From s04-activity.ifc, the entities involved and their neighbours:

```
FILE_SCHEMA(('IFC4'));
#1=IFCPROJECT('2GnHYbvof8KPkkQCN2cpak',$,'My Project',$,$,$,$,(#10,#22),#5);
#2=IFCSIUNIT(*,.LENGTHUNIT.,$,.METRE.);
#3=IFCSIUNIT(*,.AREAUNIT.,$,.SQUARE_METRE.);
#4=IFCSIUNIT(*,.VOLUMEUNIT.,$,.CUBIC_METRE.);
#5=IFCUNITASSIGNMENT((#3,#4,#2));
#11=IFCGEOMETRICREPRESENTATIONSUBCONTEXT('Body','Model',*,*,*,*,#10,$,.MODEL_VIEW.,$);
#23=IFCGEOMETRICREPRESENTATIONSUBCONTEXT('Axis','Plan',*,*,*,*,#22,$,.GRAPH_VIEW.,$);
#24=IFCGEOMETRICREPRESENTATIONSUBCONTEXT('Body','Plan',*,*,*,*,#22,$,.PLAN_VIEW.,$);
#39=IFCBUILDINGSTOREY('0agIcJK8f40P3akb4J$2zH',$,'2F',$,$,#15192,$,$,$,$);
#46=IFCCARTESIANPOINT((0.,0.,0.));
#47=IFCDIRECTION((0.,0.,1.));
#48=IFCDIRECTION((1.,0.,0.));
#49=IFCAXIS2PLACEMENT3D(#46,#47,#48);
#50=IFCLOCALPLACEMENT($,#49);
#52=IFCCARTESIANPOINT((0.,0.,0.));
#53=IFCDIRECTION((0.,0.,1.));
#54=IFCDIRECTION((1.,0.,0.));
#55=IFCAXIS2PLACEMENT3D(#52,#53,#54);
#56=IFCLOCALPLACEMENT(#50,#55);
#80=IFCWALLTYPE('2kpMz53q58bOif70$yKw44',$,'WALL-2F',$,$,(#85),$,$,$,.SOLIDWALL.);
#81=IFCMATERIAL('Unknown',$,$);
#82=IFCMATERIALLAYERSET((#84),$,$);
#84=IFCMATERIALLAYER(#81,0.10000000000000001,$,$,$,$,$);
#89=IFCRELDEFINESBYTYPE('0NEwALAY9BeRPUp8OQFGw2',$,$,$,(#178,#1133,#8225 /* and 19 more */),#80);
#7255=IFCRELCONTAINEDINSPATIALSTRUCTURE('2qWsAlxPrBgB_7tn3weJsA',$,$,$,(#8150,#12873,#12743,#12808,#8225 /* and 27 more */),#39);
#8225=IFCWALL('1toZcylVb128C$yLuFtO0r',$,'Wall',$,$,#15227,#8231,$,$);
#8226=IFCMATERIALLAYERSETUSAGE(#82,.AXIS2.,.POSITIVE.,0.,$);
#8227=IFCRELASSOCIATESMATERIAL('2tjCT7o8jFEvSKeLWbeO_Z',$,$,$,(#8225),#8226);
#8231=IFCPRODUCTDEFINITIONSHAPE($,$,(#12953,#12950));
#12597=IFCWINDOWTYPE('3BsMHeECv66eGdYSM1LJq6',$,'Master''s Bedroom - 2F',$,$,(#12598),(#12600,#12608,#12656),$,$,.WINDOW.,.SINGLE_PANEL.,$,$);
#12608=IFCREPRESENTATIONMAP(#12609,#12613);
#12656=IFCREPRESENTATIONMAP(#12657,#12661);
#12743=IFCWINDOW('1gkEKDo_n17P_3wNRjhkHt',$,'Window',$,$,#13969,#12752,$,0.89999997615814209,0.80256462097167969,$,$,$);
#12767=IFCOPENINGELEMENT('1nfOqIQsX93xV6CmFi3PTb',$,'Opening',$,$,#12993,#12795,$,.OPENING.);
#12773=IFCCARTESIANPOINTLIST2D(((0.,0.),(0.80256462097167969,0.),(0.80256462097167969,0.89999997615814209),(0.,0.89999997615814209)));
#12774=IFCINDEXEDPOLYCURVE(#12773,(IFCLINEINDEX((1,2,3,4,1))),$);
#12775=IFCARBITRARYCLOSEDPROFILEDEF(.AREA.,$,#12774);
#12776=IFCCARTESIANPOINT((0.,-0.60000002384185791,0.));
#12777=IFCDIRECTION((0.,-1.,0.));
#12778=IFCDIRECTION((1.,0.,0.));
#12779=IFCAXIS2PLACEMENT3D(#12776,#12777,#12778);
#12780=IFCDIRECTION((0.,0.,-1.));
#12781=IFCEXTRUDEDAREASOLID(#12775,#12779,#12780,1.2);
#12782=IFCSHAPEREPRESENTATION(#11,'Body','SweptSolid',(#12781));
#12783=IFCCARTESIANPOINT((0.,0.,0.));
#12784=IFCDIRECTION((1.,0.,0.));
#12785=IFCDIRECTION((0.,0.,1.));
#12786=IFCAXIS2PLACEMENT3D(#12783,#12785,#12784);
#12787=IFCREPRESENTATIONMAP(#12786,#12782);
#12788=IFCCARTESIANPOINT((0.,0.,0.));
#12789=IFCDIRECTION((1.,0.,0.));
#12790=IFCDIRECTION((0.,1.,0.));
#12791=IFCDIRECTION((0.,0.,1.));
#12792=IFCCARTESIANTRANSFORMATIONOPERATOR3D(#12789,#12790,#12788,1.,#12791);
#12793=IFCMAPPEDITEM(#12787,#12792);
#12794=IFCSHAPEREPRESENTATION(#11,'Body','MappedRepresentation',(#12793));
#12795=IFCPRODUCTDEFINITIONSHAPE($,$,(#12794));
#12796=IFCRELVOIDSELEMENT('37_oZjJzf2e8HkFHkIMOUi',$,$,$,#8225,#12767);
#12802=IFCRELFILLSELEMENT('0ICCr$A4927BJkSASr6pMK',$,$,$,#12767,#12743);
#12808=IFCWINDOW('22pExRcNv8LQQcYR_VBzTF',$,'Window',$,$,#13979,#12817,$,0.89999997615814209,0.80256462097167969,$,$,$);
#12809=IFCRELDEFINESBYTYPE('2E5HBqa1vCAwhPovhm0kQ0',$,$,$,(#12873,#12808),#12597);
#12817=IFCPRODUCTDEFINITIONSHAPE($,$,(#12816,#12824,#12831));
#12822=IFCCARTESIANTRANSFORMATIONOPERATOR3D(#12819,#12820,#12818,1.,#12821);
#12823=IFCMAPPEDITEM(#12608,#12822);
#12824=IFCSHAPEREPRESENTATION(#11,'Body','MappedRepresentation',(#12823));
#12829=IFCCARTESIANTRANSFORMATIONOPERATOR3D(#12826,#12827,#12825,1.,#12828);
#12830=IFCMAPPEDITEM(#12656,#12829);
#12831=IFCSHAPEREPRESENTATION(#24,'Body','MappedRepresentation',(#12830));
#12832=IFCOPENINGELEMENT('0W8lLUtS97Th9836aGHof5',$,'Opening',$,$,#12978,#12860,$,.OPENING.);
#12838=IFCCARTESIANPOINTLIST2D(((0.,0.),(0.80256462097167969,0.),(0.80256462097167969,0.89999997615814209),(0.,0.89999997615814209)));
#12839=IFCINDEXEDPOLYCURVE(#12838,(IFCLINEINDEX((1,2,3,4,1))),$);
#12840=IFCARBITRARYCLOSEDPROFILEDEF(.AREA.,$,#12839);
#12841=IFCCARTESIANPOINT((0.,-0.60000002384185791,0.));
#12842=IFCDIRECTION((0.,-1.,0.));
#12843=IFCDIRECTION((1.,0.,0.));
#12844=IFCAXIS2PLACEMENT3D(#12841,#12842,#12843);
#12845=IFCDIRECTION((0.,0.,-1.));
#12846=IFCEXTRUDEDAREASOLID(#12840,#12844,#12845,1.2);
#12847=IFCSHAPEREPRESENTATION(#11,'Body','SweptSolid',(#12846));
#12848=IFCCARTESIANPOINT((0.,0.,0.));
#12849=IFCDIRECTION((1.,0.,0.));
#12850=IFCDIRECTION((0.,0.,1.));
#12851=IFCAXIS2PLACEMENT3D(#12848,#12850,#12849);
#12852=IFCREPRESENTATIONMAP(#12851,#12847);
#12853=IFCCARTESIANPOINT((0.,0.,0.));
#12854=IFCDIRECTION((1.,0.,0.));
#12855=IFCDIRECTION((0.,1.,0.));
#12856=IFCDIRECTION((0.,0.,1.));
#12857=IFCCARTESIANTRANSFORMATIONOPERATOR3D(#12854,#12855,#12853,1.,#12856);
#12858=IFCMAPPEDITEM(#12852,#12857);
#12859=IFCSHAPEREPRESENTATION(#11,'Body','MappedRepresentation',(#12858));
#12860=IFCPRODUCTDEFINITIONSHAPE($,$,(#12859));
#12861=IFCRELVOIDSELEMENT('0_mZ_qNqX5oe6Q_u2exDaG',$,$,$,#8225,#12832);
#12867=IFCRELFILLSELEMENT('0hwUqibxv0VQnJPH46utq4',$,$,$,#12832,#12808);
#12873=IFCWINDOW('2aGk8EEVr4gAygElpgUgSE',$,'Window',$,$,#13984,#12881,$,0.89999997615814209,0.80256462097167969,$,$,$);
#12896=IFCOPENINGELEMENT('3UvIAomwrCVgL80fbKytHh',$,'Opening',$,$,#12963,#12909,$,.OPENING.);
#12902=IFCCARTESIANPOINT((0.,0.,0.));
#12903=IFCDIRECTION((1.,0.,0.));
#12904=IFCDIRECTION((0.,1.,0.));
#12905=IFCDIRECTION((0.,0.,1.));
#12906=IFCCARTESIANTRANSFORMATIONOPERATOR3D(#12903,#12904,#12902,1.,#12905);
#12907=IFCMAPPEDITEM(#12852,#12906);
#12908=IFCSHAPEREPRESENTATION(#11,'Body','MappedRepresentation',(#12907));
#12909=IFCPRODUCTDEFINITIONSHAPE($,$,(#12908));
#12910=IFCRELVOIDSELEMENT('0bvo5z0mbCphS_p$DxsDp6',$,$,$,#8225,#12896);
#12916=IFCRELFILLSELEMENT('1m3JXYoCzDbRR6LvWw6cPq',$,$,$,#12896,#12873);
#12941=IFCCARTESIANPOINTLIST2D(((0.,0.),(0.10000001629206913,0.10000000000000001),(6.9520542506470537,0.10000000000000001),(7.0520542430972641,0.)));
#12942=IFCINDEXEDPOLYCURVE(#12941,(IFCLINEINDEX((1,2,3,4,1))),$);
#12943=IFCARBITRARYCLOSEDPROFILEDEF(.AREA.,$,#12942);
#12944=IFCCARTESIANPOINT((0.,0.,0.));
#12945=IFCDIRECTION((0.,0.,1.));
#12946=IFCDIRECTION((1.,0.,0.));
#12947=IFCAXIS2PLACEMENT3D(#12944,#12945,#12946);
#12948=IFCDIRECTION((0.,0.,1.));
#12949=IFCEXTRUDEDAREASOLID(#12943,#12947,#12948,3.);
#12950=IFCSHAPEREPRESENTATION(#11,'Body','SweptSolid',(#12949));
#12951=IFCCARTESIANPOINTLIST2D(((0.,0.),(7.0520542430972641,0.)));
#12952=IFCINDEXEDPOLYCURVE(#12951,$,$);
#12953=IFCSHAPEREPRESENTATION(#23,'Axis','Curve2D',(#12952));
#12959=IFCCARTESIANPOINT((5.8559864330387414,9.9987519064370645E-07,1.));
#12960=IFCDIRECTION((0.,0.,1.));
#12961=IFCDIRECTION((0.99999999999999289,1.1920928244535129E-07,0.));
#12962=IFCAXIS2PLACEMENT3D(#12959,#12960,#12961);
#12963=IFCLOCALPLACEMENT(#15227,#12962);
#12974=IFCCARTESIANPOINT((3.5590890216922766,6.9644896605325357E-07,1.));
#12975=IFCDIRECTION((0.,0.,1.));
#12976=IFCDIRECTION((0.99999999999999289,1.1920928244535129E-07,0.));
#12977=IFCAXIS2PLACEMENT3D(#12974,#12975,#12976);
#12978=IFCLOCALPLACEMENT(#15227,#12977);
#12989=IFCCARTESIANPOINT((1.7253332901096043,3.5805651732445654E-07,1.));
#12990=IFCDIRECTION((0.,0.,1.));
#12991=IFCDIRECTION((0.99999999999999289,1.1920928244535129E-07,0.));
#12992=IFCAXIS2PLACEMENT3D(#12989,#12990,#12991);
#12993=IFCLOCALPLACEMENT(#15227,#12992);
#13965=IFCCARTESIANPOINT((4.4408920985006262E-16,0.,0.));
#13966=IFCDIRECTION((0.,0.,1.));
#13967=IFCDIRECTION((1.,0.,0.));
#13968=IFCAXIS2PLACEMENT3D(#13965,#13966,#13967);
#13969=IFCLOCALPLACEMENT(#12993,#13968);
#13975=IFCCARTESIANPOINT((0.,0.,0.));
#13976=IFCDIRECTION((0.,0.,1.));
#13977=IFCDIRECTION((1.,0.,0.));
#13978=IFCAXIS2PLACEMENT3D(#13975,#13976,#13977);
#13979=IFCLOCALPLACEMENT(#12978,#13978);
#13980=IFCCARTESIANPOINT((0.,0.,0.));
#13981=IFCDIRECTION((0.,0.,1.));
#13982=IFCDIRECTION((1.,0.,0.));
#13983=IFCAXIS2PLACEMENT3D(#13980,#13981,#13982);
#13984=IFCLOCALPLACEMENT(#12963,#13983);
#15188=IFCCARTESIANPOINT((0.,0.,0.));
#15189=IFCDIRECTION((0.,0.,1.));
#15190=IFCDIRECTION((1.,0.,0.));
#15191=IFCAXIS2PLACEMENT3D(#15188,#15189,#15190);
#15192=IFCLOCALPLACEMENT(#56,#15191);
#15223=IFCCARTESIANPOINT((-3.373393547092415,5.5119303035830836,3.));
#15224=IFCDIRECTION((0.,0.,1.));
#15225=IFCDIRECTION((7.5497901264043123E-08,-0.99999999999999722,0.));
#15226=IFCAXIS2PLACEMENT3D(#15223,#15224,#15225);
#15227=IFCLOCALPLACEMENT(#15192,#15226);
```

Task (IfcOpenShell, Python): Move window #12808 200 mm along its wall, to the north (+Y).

```python
import ifcopenshell
import ifcopenshell.api.geometry
import ifcopenshell.util.placement

model = ifcopenshell.open("s04-activity.ifc")

window = model.by_guid("22pExRcNv8LQQcYR_VBzTF")
opening = window.FillsVoids[0].RelatingOpeningElement
wall = opening.VoidsElements[0].RelatingBuildingElement

wall_matrix = ifcopenshell.util.placement.get_local_placement(wall.ObjectPlacement)
shift = wall_matrix[:3, 0] * -0.2
before = ifcopenshell.util.placement.get_local_placement(window.ObjectPlacement)[:3, 3].copy()

# The window is placed relative to its opening, so it follows when the opening moves.
matrix = ifcopenshell.util.placement.get_local_placement(opening.ObjectPlacement)
matrix[:3, 3] += shift
ifcopenshell.api.geometry.edit_object_placement(
    model, product=opening, matrix=matrix, is_si=False, should_transform_children=True
)

after = ifcopenshell.util.placement.get_local_placement(window.ObjectPlacement)[:3, 3]
print("window moved by", (after - before).round(3) + 0.0)

model.write("s04-activity_v2.ifc")
```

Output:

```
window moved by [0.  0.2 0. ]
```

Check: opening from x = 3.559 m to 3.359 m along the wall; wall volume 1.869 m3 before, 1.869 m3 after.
